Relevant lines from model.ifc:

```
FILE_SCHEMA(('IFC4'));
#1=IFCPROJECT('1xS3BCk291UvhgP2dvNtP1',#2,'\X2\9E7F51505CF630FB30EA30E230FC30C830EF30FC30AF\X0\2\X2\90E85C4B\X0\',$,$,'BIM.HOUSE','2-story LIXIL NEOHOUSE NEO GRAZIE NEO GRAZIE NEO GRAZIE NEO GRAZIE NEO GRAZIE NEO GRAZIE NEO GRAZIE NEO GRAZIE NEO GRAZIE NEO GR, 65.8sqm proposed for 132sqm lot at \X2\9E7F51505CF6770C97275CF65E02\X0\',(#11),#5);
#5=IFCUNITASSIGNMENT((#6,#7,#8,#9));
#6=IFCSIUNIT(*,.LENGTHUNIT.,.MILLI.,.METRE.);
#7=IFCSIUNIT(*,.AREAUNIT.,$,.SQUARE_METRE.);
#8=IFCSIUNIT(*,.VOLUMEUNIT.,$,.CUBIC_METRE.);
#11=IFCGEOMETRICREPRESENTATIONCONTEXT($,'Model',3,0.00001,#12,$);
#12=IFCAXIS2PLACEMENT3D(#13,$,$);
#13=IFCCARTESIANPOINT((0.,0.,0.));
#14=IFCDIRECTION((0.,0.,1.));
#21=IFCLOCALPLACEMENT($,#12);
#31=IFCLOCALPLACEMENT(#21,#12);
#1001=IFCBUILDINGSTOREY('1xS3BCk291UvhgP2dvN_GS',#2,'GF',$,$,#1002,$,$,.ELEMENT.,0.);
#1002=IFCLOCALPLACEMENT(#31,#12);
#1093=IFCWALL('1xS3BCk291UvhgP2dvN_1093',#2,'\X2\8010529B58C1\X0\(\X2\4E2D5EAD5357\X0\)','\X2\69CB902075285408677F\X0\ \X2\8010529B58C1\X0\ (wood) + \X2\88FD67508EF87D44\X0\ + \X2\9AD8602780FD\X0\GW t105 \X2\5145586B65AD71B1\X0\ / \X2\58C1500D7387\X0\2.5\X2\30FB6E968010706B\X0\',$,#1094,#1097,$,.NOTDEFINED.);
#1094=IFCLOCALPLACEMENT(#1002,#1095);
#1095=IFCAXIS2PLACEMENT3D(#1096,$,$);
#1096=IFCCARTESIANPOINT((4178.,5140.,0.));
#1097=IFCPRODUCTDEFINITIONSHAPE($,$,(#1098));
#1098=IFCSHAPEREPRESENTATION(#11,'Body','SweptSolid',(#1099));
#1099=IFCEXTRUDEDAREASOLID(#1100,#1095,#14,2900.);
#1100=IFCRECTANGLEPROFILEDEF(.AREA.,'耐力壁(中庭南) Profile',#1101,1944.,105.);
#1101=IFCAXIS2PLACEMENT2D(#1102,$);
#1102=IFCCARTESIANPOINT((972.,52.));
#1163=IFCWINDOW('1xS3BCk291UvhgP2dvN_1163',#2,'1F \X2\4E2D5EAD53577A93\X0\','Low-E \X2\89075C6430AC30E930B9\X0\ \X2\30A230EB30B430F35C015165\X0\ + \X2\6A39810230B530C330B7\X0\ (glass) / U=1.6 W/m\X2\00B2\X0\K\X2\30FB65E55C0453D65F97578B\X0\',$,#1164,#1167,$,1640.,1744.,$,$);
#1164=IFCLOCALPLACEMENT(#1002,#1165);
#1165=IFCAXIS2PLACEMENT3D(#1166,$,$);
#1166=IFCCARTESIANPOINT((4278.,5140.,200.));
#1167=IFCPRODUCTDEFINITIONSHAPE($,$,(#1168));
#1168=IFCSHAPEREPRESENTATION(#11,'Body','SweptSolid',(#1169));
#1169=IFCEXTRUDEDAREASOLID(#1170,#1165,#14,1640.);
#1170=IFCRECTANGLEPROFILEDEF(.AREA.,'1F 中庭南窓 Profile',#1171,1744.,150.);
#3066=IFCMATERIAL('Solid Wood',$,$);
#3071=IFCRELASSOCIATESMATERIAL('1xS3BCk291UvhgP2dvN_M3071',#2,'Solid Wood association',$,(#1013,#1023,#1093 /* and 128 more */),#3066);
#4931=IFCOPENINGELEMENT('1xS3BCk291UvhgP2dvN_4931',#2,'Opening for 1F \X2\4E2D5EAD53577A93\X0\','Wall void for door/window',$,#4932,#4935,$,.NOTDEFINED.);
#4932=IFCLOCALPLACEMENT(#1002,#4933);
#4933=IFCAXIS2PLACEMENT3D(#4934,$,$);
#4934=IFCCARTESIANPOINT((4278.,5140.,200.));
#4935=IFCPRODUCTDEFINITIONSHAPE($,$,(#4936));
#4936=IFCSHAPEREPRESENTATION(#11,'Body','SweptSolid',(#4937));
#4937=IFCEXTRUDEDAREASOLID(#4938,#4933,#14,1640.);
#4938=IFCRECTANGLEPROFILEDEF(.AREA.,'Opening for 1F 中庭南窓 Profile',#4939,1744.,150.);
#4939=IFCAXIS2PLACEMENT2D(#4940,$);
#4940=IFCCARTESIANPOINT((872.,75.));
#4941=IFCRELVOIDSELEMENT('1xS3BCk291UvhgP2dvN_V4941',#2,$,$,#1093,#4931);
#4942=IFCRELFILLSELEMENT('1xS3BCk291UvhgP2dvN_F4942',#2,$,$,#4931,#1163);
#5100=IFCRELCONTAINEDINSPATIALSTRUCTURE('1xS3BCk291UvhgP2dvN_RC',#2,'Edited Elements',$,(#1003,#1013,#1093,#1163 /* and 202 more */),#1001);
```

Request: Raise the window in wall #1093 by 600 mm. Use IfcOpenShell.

```python
import numpy as np
import ifcopenshell
import ifcopenshell.api.geometry
import ifcopenshell.util.placement
import ifcopenshell.util.unit

model = ifcopenshell.open("model.ifc")
unit_scale = ifcopenshell.util.unit.calculate_unit_scale(model)

window = model.by_guid("1xS3BCk291UvhgP2dvN_1163")
opening = window.FillsVoids[0].RelatingOpeningElement
dz = 600.0

shift = np.array([0.0, 0.0, dz])
# The window is not placed relative to its opening, so move both.
for product in (opening, window):
    matrix = ifcopenshell.util.placement.get_local_placement(product.ObjectPlacement)
    matrix[:3, 3] += shift
    ifcopenshell.api.geometry.edit_object_placement(model, product=product, matrix=matrix, is_si=False)

print(f"moved by {dz * unit_scale:+.3f} m")

model.write("model-out.ifc")
```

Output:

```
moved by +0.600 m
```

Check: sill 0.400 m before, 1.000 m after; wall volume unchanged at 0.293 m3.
